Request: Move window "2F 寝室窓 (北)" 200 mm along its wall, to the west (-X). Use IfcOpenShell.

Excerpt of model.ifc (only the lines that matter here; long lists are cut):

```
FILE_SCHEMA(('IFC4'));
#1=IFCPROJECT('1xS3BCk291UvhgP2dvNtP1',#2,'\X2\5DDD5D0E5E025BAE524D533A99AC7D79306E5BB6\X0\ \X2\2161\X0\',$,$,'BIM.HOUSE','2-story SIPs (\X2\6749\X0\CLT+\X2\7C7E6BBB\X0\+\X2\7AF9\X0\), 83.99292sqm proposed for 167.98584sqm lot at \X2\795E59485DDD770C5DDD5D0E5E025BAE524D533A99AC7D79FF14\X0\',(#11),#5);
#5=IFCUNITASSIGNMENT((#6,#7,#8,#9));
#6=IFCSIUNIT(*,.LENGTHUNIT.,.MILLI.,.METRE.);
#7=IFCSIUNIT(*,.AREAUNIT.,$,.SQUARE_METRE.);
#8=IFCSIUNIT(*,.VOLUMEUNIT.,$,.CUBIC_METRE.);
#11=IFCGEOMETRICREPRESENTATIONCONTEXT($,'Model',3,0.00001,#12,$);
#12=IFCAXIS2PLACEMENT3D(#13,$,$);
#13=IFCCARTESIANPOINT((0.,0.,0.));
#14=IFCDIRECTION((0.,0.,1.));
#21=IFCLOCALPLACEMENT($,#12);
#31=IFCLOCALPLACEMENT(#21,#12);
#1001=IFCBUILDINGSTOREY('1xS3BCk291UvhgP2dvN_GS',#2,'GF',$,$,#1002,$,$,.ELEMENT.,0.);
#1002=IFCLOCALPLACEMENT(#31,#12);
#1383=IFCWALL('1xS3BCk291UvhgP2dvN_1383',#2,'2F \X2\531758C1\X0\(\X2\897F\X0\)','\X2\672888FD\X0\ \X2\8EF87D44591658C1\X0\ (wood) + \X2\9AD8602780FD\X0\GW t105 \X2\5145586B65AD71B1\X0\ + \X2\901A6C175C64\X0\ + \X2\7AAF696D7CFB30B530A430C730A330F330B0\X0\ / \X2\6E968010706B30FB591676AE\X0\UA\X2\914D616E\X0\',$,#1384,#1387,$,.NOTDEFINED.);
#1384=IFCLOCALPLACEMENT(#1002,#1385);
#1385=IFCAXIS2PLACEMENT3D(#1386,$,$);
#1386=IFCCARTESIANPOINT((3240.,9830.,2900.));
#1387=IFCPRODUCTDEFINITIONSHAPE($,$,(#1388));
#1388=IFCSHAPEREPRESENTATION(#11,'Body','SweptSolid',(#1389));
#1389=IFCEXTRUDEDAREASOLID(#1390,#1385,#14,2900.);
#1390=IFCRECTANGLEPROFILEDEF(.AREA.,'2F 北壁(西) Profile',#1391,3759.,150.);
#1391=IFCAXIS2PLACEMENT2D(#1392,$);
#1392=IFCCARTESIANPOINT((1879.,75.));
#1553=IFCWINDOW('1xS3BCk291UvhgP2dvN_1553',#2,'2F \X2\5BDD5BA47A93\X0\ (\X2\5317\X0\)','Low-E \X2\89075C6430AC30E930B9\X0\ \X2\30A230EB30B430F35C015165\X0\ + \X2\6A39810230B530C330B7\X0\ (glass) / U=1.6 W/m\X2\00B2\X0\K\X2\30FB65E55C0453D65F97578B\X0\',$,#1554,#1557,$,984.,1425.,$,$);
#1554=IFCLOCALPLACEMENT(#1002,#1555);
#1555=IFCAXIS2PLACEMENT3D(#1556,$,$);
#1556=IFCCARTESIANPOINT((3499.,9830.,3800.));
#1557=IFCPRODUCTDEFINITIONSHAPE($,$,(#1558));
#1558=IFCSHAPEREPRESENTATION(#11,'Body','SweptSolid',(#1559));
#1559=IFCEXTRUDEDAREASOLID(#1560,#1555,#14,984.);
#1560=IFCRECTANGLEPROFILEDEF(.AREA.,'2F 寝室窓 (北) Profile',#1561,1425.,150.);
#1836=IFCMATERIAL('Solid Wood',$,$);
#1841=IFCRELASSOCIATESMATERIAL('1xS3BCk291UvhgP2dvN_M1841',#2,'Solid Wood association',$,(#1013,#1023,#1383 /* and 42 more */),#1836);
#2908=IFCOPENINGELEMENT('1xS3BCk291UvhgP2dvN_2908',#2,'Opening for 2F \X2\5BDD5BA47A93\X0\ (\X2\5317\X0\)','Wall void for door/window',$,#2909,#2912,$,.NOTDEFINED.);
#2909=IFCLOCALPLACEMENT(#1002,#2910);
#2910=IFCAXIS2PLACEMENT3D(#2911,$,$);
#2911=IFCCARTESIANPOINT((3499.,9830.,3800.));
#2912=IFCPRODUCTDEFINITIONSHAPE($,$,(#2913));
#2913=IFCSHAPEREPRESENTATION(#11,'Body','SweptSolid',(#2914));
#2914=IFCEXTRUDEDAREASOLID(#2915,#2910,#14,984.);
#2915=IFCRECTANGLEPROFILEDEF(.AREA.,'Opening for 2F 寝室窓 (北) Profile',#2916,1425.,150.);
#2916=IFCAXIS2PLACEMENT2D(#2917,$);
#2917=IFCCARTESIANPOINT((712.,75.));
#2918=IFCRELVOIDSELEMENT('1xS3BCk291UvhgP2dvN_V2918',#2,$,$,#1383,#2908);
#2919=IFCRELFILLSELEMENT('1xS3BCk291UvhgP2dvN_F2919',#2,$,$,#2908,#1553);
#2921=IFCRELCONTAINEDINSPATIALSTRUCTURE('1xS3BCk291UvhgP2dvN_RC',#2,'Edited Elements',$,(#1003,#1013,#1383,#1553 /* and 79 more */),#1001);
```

```python
import ifcopenshell
import ifcopenshell.api.geometry
import ifcopenshell.util.placement
import ifcopenshell.util.unit

model = ifcopenshell.open("model.ifc")
unit_scale = ifcopenshell.util.unit.calculate_unit_scale(model)

window = model.by_guid("1xS3BCk291UvhgP2dvN_1553")
opening = window.FillsVoids[0].RelatingOpeningElement
wall = opening.VoidsElements[0].RelatingBuildingElement

wall_matrix = ifcopenshell.util.placement.get_local_placement(wall.ObjectPlacement)
shift = wall_matrix[:3, 0] * -0.2 / unit_scale
before = ifcopenshell.util.placement.get_local_placement(window.ObjectPlacement)[:3, 3].copy()

# The window is not placed relative to its opening, so move both.
for product in (opening, window):
    matrix = ifcopenshell.util.placement.get_local_placement(product.ObjectPlacement)
    matrix[:3, 3] += shift
    ifcopenshell.api.geometry.edit_object_placement(model, product=product, matrix=matrix, is_si=False)

after = ifcopenshell.util.placement.get_local_placement(window.ObjectPlacement)[:3, 3]
print("window moved by", (after - before).round(3) + 0.0)

model.write("model_updated.ifc")
```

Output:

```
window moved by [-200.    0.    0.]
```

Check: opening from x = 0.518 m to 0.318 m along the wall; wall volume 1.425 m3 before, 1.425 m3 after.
